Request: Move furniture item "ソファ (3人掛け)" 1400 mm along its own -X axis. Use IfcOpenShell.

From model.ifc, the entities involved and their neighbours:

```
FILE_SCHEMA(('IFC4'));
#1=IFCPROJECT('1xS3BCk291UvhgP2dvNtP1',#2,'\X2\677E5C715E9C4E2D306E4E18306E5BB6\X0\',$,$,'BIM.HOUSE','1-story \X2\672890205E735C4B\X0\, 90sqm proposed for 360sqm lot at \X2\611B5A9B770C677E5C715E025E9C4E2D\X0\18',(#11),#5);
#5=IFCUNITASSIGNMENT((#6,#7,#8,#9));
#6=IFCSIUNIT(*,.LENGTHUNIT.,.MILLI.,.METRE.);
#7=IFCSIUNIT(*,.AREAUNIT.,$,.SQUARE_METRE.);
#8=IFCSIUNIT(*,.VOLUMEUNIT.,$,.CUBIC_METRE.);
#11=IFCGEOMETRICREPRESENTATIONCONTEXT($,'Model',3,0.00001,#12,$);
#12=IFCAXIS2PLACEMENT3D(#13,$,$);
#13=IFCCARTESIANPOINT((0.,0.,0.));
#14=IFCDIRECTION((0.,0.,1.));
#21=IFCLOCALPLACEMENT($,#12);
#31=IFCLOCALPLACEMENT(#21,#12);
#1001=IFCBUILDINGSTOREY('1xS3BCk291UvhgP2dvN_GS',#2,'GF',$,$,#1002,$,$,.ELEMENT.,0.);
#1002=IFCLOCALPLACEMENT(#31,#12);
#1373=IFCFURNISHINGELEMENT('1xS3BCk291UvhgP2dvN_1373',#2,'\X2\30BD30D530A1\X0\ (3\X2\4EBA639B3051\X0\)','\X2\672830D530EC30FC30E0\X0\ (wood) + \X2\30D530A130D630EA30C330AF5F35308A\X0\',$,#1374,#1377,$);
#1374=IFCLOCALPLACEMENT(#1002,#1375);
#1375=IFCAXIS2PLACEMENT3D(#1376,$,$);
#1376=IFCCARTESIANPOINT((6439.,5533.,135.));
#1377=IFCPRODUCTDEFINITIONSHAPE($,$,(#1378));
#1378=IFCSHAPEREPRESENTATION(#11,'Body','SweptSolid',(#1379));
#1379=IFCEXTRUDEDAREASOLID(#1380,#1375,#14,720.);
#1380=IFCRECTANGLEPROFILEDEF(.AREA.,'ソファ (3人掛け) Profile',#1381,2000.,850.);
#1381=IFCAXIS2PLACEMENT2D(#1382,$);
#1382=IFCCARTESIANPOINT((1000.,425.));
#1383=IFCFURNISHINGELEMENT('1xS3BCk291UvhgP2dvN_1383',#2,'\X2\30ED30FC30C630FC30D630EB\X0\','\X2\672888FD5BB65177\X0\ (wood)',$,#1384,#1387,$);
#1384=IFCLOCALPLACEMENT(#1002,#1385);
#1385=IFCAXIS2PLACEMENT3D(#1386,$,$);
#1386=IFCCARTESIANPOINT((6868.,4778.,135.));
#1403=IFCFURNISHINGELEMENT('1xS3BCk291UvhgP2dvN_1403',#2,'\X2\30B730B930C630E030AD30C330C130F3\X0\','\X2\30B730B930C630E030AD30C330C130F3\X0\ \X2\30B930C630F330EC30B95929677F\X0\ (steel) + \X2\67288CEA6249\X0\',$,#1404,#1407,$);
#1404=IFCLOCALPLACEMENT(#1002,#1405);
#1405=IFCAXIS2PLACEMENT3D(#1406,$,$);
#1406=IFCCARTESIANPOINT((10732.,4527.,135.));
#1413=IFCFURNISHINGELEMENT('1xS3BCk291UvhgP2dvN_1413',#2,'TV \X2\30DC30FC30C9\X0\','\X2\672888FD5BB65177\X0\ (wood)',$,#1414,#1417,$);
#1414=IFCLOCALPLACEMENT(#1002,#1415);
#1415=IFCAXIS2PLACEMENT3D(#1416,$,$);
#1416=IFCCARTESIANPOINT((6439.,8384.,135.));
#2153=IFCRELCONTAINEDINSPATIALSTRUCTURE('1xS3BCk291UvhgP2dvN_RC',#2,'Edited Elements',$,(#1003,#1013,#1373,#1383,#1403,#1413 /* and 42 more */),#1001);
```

```python
import ifcopenshell
import ifcopenshell.api.geometry
import ifcopenshell.util.placement

model = ifcopenshell.open("model.ifc")

item = model.by_guid("1xS3BCk291UvhgP2dvN_1373")
matrix = ifcopenshell.util.placement.get_local_placement(item.ObjectPlacement)
matrix[:3, 3] -= matrix[:3, 0] * 1400.0
ifcopenshell.api.geometry.edit_object_placement(model, product=item, matrix=matrix, is_si=False)

print(ifcopenshell.util.placement.get_local_placement(item.ObjectPlacement).round(3) + 0.0)

model.write("model_updated.ifc")
```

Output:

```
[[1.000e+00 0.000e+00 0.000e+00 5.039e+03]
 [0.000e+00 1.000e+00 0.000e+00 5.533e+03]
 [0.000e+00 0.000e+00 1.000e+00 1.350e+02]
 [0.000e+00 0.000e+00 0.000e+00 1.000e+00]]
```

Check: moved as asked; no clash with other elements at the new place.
